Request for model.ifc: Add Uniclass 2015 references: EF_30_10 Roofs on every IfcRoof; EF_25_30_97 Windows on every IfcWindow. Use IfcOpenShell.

First a look at what the model holds.

```python
import ifcopenshell

model = ifcopenshell.open("model.ifc")
print(model.schema)
print("classifications:", [c.Name for c in model.by_type("IfcClassification")])
for ifc_class in ("IfcDoor", "IfcRoof", "IfcStair", "IfcWall", "IfcWindow"):
    print(ifc_class, len(model.by_type(ifc_class)))
```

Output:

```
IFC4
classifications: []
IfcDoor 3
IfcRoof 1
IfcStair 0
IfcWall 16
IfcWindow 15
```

```python
import ifcopenshell
import ifcopenshell.api.classification

model = ifcopenshell.open("model.ifc")

system = ifcopenshell.api.classification.add_classification(model, classification="Uniclass 2015")

codes = {
    "IfcRoof": ("EF_30_10", "Roofs"),
    "IfcWindow": ("EF_25_30_97", "Windows"),
}
for ifc_class, (code, name) in codes.items():
    products = model.by_type(ifc_class)
    ifcopenshell.api.classification.add_reference(
        model, products=products, classification=system, identification=code, name=name
    )
    print(code, len(products))

model.write("model_rev.ifc")
```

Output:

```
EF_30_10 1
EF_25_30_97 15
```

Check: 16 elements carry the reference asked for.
